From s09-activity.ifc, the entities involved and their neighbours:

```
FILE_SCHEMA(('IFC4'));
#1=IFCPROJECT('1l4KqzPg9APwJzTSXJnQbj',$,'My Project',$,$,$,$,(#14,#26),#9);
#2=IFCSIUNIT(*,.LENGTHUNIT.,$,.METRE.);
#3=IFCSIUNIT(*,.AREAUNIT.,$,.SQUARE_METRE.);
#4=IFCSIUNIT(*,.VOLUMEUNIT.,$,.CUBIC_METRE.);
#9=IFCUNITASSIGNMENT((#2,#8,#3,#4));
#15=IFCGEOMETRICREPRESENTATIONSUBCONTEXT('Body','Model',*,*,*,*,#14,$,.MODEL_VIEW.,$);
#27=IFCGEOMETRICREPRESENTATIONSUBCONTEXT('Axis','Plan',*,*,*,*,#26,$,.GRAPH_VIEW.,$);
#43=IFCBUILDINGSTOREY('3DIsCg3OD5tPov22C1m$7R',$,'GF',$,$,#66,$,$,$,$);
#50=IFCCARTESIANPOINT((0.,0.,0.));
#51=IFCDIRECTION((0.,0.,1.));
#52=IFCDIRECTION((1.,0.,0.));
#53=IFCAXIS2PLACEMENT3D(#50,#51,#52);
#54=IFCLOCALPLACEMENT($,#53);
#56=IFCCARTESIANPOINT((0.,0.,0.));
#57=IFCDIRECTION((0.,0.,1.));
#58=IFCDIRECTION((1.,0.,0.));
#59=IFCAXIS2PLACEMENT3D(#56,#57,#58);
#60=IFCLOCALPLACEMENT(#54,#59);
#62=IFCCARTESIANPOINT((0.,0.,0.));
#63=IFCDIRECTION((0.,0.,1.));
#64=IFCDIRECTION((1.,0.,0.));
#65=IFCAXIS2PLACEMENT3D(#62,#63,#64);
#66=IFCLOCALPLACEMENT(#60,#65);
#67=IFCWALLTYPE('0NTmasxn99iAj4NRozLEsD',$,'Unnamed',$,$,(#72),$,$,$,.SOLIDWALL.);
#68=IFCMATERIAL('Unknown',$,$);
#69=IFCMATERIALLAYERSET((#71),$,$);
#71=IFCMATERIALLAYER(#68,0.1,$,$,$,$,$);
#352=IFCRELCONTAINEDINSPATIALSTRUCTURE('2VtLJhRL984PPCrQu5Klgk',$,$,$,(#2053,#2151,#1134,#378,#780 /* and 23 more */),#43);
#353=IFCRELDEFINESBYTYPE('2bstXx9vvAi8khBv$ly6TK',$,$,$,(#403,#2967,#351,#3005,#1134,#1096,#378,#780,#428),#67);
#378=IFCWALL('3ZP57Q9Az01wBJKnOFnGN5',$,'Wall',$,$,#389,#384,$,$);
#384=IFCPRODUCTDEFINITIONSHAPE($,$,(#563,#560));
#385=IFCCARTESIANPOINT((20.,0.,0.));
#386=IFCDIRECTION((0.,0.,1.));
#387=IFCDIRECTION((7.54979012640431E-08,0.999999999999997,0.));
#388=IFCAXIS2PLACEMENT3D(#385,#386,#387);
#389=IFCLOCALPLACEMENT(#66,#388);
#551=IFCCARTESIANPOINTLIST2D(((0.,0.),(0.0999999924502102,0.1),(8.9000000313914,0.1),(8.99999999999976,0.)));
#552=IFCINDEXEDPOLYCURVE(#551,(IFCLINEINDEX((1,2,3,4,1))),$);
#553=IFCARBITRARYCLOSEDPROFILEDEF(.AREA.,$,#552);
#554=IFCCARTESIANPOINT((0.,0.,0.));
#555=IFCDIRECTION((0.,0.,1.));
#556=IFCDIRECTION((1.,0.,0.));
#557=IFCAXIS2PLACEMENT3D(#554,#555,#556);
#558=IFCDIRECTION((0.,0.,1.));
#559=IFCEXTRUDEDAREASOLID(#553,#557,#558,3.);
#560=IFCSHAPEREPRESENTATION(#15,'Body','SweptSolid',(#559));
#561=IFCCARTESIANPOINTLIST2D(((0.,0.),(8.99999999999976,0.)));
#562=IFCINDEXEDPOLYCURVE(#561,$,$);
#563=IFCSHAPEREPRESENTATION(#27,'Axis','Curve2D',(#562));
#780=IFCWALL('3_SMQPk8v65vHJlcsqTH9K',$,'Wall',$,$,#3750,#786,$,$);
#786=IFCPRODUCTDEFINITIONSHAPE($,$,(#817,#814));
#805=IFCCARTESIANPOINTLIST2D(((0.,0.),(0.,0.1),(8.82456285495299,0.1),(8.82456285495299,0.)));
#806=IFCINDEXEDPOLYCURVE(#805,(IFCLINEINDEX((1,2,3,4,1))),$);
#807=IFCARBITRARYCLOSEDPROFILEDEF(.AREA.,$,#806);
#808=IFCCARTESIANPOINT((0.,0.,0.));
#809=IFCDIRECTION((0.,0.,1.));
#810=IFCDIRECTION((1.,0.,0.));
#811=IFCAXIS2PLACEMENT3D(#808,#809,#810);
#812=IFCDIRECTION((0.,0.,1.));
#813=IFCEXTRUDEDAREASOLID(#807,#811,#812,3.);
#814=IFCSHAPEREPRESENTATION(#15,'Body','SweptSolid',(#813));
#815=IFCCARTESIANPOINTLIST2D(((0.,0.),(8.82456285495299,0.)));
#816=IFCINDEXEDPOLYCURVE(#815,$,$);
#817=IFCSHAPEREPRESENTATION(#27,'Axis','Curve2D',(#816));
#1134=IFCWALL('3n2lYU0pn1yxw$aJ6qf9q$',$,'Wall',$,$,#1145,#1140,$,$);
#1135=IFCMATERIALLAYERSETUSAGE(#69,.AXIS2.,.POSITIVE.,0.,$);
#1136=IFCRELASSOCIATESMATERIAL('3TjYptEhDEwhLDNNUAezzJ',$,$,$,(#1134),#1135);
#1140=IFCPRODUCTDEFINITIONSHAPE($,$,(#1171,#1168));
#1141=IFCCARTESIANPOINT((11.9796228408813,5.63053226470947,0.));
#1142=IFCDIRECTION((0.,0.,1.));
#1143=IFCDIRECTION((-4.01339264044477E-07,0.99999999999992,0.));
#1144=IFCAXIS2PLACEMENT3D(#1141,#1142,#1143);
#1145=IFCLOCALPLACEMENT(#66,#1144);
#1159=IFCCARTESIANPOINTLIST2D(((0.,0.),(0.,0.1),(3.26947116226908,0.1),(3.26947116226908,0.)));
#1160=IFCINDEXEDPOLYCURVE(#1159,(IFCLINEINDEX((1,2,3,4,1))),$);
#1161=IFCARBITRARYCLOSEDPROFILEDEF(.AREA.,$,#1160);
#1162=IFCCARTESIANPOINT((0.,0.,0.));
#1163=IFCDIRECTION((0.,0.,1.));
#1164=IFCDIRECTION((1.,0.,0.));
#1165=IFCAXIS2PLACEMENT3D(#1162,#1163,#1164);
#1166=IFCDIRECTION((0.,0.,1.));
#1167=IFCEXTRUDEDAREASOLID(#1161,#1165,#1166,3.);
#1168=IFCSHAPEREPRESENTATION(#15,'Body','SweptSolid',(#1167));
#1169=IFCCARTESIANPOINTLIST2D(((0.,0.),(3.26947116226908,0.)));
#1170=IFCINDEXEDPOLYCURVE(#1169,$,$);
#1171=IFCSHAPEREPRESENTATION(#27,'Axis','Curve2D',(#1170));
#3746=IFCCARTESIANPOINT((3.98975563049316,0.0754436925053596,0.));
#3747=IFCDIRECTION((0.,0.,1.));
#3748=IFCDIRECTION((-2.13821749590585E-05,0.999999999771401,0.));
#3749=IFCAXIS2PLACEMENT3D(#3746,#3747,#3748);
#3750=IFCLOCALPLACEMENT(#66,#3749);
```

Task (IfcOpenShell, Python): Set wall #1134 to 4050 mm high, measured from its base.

```python
import ifcopenshell
import ifcopenshell.geom
import ifcopenshell.util.representation
import ifcopenshell.util.shape
import ifcopenshell.util.unit

model = ifcopenshell.open("s09-activity.ifc")
unit_scale = ifcopenshell.util.unit.calculate_unit_scale(model)
settings = ifcopenshell.geom.settings()


def volume(element):
    """Net volume in cubic metres, openings subtracted."""
    shape = ifcopenshell.geom.create_shape(settings, element)
    return ifcopenshell.util.shape.get_volume(shape.geometry)


wall = model.by_guid("3n2lYU0pn1yxw$aJ6qf9q$")
before = volume(wall)

body = ifcopenshell.util.representation.get_representation(wall, "Model", "Body")
solid = body.Items[0]
old_height = solid.Depth
solid.Depth = 4.05 / unit_scale
after = volume(wall)

print(f"height {old_height:g} -> {solid.Depth:g}, volume {before:.3f} -> {after:.3f} m3")

model.write("s09-activity_updated.ifc")
```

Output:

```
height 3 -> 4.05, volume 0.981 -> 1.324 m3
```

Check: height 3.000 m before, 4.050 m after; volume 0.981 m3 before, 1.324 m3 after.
